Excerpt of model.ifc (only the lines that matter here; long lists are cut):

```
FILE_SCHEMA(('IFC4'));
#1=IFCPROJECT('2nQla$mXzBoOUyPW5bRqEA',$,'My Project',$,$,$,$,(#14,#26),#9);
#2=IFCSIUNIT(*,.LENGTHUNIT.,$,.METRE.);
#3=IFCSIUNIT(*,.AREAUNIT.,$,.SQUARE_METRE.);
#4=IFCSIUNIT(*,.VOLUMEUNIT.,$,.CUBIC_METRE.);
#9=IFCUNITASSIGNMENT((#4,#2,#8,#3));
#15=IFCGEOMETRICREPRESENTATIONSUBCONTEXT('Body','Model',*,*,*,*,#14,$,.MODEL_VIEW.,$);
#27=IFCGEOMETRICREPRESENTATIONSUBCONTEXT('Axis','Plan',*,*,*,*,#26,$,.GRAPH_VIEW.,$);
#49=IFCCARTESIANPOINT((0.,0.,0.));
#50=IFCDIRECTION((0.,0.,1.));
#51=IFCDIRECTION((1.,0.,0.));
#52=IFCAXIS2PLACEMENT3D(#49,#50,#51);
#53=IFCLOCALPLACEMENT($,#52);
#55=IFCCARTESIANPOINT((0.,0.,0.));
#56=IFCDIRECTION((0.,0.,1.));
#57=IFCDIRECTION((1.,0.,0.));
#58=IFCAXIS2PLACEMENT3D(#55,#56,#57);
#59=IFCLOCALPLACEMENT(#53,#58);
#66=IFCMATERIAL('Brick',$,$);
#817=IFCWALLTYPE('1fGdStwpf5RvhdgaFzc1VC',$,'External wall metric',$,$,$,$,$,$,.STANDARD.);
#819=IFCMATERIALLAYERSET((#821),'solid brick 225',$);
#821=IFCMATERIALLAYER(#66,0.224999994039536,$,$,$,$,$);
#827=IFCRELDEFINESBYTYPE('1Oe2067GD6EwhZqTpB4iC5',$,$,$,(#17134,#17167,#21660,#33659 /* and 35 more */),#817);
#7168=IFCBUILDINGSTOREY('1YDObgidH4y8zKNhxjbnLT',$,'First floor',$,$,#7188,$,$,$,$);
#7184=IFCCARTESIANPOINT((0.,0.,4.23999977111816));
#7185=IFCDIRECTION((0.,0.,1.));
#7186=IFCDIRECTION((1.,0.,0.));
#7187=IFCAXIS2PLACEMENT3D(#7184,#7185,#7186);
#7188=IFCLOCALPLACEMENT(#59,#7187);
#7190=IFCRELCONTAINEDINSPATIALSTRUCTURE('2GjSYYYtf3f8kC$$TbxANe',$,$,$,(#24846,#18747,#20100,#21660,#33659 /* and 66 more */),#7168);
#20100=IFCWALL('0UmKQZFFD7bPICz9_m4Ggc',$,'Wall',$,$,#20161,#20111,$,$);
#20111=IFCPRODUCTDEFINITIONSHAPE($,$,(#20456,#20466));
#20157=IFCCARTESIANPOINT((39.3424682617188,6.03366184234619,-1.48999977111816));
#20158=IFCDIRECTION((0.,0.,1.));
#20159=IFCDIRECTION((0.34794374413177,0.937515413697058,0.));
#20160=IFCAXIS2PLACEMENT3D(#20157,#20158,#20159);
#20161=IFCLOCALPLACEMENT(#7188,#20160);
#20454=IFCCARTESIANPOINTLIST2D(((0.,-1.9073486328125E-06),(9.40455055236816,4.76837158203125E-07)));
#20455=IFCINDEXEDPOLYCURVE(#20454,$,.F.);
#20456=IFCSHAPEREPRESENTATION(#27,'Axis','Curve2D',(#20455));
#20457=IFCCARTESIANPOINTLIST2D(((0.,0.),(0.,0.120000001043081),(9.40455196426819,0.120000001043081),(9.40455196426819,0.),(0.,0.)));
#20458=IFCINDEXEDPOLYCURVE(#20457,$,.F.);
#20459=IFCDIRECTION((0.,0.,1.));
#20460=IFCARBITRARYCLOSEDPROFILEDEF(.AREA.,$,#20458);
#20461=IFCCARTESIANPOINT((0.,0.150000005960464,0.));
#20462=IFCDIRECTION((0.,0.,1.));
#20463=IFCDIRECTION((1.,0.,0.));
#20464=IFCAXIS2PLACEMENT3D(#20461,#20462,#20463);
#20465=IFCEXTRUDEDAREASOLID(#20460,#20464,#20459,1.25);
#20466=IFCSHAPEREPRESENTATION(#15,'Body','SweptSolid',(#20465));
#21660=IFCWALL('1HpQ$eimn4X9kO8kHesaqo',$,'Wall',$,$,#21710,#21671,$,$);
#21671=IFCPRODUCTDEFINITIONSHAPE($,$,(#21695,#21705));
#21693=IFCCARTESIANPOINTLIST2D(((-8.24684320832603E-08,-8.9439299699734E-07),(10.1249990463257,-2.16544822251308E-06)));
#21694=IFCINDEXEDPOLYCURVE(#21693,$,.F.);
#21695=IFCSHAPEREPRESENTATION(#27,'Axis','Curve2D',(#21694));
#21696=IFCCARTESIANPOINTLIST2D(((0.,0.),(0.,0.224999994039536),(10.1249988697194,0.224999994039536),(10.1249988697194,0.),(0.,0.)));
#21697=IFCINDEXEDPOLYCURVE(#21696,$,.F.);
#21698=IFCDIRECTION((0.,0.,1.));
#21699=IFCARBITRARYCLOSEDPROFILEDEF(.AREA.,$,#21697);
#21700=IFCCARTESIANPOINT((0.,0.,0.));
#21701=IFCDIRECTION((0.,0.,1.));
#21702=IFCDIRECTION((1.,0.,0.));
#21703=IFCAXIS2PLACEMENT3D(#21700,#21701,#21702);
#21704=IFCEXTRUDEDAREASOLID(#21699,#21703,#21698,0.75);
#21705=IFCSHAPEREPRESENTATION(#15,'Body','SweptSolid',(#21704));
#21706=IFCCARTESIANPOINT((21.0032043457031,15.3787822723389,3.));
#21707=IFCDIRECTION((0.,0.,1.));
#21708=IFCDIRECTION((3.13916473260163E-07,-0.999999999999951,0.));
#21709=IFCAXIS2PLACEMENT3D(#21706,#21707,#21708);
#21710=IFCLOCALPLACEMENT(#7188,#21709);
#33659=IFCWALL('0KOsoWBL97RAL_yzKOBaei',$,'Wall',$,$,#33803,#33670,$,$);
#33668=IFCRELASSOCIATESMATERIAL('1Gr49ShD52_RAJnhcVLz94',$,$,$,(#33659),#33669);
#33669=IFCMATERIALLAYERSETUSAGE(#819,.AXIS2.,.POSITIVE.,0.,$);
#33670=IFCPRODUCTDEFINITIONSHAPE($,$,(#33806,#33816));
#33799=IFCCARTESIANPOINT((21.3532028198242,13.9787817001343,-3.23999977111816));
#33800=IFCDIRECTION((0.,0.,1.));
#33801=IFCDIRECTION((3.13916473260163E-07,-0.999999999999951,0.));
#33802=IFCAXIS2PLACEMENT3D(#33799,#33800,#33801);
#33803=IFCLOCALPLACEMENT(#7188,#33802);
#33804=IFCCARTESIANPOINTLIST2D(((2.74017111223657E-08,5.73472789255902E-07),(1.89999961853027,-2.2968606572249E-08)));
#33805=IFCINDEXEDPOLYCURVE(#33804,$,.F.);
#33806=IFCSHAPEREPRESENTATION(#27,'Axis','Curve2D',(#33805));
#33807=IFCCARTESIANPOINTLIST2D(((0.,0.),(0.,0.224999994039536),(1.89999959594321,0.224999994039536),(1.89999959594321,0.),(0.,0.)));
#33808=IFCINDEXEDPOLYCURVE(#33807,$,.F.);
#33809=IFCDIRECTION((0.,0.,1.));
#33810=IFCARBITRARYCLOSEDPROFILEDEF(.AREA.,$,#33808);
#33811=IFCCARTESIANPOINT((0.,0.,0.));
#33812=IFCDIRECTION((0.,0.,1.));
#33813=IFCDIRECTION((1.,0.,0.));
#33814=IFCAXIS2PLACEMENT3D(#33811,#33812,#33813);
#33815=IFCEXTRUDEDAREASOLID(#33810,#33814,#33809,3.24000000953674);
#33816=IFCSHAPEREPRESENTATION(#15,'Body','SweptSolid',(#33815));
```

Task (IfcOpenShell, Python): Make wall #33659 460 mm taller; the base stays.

```python
import ifcopenshell
import ifcopenshell.geom
import ifcopenshell.util.representation
import ifcopenshell.util.shape
import ifcopenshell.util.unit

model = ifcopenshell.open("model.ifc")
unit_scale = ifcopenshell.util.unit.calculate_unit_scale(model)
settings = ifcopenshell.geom.settings()


def volume(element):
    """Net volume in cubic metres, openings subtracted."""
    shape = ifcopenshell.geom.create_shape(settings, element)
    return ifcopenshell.util.shape.get_volume(shape.geometry)


wall = model.by_id(33659)
before = volume(wall)

body = ifcopenshell.util.representation.get_representation(wall, "Model", "Body")
solid = body.Items[0]
old_height = solid.Depth
solid.Depth += 0.46 / unit_scale
after = volume(wall)

print(f"height {old_height:g} -> {solid.Depth:g}, volume {before:.3f} -> {after:.3f} m3")

model.write("model_v2.ifc")
```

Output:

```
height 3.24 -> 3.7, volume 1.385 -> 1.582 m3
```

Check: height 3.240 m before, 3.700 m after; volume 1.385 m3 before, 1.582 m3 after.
